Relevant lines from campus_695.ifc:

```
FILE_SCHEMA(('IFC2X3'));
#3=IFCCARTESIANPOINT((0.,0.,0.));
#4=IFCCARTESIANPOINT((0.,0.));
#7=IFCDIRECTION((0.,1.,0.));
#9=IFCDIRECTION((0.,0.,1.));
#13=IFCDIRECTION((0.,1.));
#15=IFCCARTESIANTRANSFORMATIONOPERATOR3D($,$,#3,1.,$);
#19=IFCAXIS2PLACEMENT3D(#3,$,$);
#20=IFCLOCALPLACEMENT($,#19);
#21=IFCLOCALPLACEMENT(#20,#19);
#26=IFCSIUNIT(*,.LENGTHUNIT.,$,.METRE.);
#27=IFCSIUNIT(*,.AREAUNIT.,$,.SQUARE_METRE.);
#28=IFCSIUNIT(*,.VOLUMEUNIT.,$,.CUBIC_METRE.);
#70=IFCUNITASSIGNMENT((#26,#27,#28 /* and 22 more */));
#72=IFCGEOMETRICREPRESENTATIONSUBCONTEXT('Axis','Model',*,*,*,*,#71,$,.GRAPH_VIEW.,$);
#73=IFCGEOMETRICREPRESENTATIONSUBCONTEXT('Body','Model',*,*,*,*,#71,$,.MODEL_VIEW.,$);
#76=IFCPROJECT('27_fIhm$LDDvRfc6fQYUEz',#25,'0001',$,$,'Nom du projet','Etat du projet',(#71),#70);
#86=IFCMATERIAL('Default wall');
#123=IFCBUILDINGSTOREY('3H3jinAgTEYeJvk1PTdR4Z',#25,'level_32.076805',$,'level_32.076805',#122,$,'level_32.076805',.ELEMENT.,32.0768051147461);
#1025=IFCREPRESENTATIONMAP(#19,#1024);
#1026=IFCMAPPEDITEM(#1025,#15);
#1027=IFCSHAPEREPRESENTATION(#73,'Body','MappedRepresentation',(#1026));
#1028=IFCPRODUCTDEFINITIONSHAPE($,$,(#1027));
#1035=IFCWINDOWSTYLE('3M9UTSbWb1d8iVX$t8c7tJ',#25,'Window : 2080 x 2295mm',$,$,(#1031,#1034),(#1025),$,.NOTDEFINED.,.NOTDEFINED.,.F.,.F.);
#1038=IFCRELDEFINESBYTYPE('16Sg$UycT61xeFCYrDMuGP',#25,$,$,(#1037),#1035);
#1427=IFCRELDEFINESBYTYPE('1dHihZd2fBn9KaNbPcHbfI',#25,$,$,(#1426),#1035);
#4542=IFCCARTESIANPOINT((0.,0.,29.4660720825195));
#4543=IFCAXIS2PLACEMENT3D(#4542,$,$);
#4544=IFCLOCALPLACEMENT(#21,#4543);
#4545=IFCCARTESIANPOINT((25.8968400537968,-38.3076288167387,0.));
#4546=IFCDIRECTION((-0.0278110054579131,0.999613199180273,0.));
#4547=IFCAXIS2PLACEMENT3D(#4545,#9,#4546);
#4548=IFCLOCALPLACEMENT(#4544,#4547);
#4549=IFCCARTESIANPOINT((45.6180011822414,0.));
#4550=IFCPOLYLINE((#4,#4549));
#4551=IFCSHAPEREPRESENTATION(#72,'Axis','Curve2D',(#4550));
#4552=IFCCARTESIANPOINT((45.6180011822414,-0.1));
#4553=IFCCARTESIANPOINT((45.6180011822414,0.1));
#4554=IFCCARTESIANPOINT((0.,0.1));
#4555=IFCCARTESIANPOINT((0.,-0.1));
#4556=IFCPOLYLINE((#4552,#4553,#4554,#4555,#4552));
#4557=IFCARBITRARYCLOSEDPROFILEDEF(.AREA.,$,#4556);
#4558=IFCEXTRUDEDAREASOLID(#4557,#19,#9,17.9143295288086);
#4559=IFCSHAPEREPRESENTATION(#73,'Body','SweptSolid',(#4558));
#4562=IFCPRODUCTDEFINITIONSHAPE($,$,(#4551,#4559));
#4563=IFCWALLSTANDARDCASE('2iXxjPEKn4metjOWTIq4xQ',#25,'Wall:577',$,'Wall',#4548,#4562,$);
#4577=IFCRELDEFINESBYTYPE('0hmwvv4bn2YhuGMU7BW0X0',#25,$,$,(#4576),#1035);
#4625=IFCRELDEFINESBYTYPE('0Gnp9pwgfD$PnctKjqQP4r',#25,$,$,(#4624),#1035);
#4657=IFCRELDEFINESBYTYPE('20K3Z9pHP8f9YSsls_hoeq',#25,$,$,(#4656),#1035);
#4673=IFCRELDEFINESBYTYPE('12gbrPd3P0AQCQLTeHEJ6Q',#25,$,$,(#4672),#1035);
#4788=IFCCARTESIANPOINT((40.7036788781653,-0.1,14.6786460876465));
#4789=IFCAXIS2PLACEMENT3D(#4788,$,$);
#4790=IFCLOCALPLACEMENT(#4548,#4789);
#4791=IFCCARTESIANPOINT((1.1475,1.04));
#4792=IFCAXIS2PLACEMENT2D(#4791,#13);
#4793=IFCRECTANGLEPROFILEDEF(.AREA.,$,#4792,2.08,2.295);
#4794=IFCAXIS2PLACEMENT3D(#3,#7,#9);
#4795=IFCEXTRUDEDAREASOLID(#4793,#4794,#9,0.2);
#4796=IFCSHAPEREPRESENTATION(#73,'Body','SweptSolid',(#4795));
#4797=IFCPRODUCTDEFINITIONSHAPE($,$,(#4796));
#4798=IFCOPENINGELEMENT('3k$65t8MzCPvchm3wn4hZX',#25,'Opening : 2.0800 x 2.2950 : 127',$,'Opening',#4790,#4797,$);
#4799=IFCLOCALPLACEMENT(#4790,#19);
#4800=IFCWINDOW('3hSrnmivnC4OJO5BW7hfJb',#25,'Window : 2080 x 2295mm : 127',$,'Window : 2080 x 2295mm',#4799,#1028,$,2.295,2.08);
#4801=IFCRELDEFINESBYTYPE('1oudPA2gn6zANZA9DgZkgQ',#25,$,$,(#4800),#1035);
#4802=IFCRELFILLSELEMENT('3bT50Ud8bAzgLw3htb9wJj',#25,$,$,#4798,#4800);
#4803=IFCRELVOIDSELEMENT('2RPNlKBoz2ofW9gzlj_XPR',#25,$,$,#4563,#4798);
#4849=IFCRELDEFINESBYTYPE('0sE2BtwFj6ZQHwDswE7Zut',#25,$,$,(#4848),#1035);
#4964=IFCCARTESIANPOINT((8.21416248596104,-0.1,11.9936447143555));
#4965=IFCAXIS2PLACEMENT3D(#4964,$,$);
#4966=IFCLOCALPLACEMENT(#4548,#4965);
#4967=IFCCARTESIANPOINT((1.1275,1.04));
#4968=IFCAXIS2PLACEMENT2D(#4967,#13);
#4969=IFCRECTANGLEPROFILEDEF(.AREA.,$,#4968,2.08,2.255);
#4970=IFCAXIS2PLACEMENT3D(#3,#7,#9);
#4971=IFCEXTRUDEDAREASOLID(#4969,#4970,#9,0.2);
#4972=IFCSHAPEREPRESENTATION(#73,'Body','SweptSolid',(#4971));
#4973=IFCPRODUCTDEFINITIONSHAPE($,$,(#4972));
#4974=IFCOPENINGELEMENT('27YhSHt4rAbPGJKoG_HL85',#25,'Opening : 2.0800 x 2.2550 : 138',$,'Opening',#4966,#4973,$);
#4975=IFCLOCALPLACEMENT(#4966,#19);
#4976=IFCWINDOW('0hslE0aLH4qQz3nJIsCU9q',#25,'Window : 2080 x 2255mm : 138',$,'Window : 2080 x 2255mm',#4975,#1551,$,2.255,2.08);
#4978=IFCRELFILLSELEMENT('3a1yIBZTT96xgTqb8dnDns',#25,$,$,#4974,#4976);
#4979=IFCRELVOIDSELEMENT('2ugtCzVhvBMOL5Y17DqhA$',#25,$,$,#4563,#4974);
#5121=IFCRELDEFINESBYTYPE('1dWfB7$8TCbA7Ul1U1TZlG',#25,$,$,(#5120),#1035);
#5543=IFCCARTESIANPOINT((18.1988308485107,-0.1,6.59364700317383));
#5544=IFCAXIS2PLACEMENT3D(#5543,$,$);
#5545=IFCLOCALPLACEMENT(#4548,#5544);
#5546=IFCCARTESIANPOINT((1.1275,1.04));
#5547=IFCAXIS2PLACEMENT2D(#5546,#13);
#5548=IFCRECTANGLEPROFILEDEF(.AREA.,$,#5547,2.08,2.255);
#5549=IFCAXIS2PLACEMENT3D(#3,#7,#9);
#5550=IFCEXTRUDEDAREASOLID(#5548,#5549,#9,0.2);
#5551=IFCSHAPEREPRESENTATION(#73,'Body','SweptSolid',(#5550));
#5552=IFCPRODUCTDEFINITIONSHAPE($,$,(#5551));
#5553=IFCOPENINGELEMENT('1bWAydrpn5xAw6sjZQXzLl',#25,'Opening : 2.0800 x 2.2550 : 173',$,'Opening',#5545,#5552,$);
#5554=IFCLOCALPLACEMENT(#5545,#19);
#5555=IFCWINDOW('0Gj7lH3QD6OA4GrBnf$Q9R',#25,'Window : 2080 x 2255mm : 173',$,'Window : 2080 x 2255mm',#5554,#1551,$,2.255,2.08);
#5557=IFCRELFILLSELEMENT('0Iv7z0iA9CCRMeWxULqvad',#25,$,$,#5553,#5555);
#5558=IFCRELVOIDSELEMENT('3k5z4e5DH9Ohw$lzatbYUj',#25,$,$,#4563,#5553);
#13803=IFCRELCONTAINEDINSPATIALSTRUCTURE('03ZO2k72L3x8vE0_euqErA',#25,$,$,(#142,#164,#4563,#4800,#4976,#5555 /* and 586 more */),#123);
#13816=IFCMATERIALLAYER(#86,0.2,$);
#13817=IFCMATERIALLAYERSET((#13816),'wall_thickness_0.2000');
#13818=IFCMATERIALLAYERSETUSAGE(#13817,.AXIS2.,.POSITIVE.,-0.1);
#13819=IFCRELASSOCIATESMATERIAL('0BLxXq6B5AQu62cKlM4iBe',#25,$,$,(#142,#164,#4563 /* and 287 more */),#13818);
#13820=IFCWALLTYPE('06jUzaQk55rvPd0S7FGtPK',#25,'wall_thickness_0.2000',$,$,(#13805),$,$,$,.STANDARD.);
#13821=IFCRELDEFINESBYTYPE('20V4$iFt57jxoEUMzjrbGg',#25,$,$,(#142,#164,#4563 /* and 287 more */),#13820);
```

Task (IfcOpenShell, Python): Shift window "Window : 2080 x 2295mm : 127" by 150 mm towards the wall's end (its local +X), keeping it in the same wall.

```python
import ifcopenshell
import ifcopenshell.api.geometry
import ifcopenshell.util.placement
import ifcopenshell.util.unit

model = ifcopenshell.open("campus_695.ifc")
unit_scale = ifcopenshell.util.unit.calculate_unit_scale(model)

window = model.by_guid("3hSrnmivnC4OJO5BW7hfJb")
opening = window.FillsVoids[0].RelatingOpeningElement
wall = opening.VoidsElements[0].RelatingBuildingElement

wall_matrix = ifcopenshell.util.placement.get_local_placement(wall.ObjectPlacement)
shift = wall_matrix[:3, 0] * 0.15 / unit_scale
before = ifcopenshell.util.placement.get_local_placement(window.ObjectPlacement)[:3, 3].copy()

# The window is placed relative to its opening, so it follows when the opening moves.
matrix = ifcopenshell.util.placement.get_local_placement(opening.ObjectPlacement)
matrix[:3, 3] += shift
ifcopenshell.api.geometry.edit_object_placement(
    model, product=opening, matrix=matrix, is_si=False, should_transform_children=True
)

after = ifcopenshell.util.placement.get_local_placement(window.ObjectPlacement)[:3, 3]
print("window moved by", (after - before).round(3) + 0.0)

model.write("campus_695_updated.ifc")
```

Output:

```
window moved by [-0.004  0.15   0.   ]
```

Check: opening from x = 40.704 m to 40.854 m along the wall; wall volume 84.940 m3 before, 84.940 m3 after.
